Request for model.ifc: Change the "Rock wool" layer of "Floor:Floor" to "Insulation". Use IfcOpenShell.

First a look at what the model holds.

```python
import ifcopenshell
import ifcopenshell.util.element

model = ifcopenshell.open("model.ifc")
print(model.schema)
for layer_set in model.by_type("IfcMaterialLayerSet"):
    if layer_set.LayerSetName == "Floor:Floor":
        for layer in layer_set.MaterialLayers:
            print(layer.id(), layer.Material and layer.Material.Name, layer.LayerThickness, sep=" | ")
        print(len(ifcopenshell.util.element.get_elements_by_material(model, layer_set)), "elements and types use it")
print(sorted(m.Name for m in model.by_type("IfcMaterial") if m.Name)[:60])
```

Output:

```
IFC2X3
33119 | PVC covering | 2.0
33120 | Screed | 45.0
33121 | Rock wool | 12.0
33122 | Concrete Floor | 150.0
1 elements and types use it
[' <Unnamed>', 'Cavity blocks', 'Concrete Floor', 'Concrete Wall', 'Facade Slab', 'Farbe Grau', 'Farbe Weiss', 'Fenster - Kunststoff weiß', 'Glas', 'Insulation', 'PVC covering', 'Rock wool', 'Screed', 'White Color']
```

```python
import ifcopenshell
import ifcopenshell.api.material

model = ifcopenshell.open("model.ifc")

layer_set = next(s for s in model.by_type("IfcMaterialLayerSet") if s.LayerSetName == "Floor:Floor")
layer = next(l for l in layer_set.MaterialLayers if l.Material and l.Material.Name == "Rock wool")
material = next(m for m in model.by_type("IfcMaterial") if m.Name == "Insulation")

# Point this one layer at the other material; renaming the old one would change it everywhere.
ifcopenshell.api.material.edit_layer(model, layer=layer, attributes={}, material=material)

print([l.Material.Name if l.Material else None for l in layer_set.MaterialLayers])

model.write("model_edited.ifc")
```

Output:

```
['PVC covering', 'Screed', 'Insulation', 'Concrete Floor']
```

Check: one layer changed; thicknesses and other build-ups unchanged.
